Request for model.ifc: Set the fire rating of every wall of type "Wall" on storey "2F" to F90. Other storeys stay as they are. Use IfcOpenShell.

First a look at what the model holds.

```python
import ifcopenshell
import ifcopenshell.util.element

model = ifcopenshell.open("model.ifc")
print(model.schema)
storey = next(s for s in model.by_type("IfcBuildingStorey") if s.Name == "2F")
walls = [e for e in ifcopenshell.util.element.get_decomposition(storey) if e.is_a("IfcWall")]
seen = {}
for e in walls:
    element_type = ifcopenshell.util.element.get_type(e)
    key = (element_type.Name if element_type != e and element_type else None, ifcopenshell.util.element.get_pset(e, "Pset_WallCommon", "FireRating"))
    seen[key] = seen.get(key, 0) + 1
for (name, value), count in sorted(seen.items(), key=str):
    print(count, "x", name, "|", value)
```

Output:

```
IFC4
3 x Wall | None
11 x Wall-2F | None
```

```python
import ifcopenshell
import ifcopenshell.api.pset
import ifcopenshell.util.element

model = ifcopenshell.open("model.ifc")

storey = next(s for s in model.by_type("IfcBuildingStorey") if s.Name == "2F")
walls = [e for e in ifcopenshell.util.element.get_decomposition(storey) if e.is_a("IfcWall")]

count = 0
for e in walls:
    element_type = ifcopenshell.util.element.get_type(e)
    if element_type in (None, e) or element_type.Name != "Wall":
        continue
    # add_pset returns the element's existing set when there is one.
    pset = ifcopenshell.api.pset.add_pset(model, product=e, name="Pset_WallCommon")
    ifcopenshell.api.pset.edit_pset(model, pset=pset, properties={"FireRating": "F90"})
    count += 1

print(count, "walls updated")

model.write("model_v2.ifc")
```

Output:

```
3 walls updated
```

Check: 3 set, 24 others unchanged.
